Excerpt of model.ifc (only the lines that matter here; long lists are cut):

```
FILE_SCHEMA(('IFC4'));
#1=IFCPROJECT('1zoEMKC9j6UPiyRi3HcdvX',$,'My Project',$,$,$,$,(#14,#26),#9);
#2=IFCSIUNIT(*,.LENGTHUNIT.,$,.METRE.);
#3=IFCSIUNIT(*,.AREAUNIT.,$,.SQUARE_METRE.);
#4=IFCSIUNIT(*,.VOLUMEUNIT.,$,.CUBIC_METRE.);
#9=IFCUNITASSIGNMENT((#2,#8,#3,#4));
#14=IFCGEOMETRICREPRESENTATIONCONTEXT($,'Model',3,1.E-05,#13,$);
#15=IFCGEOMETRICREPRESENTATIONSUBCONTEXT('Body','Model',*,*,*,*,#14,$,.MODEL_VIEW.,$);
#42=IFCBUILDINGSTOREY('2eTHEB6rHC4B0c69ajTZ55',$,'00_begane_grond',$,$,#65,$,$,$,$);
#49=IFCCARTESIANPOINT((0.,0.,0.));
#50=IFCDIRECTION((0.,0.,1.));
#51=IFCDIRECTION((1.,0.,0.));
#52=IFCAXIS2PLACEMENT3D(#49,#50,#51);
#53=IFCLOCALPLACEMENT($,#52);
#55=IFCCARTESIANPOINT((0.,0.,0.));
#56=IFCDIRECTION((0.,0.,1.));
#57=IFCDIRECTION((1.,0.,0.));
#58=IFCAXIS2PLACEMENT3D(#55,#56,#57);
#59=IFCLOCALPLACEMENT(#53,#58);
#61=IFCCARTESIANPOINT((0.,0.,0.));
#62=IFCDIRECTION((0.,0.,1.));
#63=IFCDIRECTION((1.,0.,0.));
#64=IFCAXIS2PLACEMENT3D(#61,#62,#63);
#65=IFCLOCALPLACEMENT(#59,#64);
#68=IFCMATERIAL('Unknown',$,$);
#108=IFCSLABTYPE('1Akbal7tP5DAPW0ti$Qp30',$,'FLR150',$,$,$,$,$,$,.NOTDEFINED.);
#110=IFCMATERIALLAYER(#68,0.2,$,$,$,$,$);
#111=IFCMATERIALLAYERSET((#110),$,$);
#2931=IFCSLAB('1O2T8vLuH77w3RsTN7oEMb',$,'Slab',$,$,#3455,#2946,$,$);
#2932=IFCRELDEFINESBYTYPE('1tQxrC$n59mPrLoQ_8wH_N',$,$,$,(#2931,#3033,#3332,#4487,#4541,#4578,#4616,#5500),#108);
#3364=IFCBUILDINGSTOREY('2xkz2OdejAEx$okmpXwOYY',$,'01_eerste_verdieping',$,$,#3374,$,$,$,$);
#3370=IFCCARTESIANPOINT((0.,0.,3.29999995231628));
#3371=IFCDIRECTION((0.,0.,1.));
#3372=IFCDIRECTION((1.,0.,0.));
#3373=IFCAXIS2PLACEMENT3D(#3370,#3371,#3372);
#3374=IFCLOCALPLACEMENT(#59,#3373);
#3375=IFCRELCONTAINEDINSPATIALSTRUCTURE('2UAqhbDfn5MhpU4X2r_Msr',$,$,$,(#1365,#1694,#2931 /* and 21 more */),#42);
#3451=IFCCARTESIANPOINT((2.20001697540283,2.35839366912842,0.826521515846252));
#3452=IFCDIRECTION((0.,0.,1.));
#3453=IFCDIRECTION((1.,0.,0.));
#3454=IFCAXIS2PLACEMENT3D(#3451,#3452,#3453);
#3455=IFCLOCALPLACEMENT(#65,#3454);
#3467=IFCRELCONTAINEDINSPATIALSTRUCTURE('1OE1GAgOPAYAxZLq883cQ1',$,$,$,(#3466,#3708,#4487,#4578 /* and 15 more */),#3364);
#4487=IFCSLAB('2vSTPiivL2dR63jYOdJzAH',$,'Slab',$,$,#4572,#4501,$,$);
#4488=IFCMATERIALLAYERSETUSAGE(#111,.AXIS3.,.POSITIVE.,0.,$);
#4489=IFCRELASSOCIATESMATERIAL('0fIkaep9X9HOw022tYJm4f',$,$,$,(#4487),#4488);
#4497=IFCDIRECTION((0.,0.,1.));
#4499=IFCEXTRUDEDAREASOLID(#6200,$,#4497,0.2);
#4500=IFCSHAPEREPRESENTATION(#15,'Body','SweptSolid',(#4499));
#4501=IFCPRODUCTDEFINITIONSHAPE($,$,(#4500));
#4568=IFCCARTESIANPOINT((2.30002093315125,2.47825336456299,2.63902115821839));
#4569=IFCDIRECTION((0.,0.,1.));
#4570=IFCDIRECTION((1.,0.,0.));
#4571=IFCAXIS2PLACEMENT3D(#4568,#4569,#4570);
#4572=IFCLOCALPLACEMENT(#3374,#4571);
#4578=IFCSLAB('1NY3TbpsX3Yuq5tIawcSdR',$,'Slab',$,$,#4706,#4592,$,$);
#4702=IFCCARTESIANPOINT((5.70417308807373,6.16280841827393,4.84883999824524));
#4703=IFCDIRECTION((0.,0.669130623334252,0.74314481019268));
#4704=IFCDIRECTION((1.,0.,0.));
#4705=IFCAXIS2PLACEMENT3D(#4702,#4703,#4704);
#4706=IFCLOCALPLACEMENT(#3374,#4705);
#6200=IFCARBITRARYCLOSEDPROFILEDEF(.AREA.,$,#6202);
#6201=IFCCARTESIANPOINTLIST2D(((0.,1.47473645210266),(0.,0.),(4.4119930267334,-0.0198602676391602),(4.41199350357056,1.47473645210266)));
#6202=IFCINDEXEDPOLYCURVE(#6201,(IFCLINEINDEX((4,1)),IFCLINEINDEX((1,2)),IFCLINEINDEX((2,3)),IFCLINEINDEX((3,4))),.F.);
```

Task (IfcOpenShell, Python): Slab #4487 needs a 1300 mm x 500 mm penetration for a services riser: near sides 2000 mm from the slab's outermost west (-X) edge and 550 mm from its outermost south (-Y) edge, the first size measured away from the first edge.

```python
import numpy as np
import ifcopenshell
import ifcopenshell.api.feature
import ifcopenshell.api.geometry
import ifcopenshell.api.root
import ifcopenshell.geom
import ifcopenshell.util.placement
import ifcopenshell.util.representation
import ifcopenshell.util.shape
import ifcopenshell.util.unit

model = ifcopenshell.open("model.ifc")
unit_scale = ifcopenshell.util.unit.calculate_unit_scale(model)
settings = ifcopenshell.geom.settings()


def volume(element):
    """Net volume in cubic metres, openings subtracted."""
    shape = ifcopenshell.geom.create_shape(settings, element)
    return ifcopenshell.util.shape.get_volume(shape.geometry)


slab = model.by_id(4487)
before = volume(slab)

# Extent in the slab's own axes, in metres. The edges named are its -X and -Y sides.
slab_shape = ifcopenshell.geom.create_shape(settings, slab)
vertices = ifcopenshell.util.shape.get_vertices(slab_shape.geometry)
x_min, y_min, bottom = vertices.min(axis=0)
top = vertices[:, 2].max()

opening = ifcopenshell.api.root.create_entity(model, ifc_class="IfcOpeningElement", name="Services riser opening", predefined_type="OPENING")
context = ifcopenshell.util.representation.get_context(model, "Model", "Body", "MODEL_VIEW")
width, depth = 1.3, 0.5
outline = [(0.0, 0.0), (width, 0.0), (width, depth), (0.0, depth), (0.0, 0.0)]
# Overshoot both faces by 50 mm so the cut is clean.
shape = ifcopenshell.api.geometry.add_slab_representation(
    model, context=context, depth=top - bottom + 0.1, polyline=outline
)
ifcopenshell.api.geometry.assign_representation(model, product=opening, representation=shape)

matrix = ifcopenshell.util.placement.get_local_placement(slab.ObjectPlacement)
matrix[:, 3] = matrix @ np.append(np.array([x_min + 2, y_min + 0.55, bottom - 0.05]) / unit_scale, 1.0)
ifcopenshell.api.geometry.edit_object_placement(model, product=opening, matrix=matrix, is_si=False)
ifcopenshell.api.feature.add_feature(model, feature=opening, element=slab)

after = volume(slab)

print(f"slab volume {before:.3f} -> {after:.3f} m3")

model.write("model_updated.ifc")
```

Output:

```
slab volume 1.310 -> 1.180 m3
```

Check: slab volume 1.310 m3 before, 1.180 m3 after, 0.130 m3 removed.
